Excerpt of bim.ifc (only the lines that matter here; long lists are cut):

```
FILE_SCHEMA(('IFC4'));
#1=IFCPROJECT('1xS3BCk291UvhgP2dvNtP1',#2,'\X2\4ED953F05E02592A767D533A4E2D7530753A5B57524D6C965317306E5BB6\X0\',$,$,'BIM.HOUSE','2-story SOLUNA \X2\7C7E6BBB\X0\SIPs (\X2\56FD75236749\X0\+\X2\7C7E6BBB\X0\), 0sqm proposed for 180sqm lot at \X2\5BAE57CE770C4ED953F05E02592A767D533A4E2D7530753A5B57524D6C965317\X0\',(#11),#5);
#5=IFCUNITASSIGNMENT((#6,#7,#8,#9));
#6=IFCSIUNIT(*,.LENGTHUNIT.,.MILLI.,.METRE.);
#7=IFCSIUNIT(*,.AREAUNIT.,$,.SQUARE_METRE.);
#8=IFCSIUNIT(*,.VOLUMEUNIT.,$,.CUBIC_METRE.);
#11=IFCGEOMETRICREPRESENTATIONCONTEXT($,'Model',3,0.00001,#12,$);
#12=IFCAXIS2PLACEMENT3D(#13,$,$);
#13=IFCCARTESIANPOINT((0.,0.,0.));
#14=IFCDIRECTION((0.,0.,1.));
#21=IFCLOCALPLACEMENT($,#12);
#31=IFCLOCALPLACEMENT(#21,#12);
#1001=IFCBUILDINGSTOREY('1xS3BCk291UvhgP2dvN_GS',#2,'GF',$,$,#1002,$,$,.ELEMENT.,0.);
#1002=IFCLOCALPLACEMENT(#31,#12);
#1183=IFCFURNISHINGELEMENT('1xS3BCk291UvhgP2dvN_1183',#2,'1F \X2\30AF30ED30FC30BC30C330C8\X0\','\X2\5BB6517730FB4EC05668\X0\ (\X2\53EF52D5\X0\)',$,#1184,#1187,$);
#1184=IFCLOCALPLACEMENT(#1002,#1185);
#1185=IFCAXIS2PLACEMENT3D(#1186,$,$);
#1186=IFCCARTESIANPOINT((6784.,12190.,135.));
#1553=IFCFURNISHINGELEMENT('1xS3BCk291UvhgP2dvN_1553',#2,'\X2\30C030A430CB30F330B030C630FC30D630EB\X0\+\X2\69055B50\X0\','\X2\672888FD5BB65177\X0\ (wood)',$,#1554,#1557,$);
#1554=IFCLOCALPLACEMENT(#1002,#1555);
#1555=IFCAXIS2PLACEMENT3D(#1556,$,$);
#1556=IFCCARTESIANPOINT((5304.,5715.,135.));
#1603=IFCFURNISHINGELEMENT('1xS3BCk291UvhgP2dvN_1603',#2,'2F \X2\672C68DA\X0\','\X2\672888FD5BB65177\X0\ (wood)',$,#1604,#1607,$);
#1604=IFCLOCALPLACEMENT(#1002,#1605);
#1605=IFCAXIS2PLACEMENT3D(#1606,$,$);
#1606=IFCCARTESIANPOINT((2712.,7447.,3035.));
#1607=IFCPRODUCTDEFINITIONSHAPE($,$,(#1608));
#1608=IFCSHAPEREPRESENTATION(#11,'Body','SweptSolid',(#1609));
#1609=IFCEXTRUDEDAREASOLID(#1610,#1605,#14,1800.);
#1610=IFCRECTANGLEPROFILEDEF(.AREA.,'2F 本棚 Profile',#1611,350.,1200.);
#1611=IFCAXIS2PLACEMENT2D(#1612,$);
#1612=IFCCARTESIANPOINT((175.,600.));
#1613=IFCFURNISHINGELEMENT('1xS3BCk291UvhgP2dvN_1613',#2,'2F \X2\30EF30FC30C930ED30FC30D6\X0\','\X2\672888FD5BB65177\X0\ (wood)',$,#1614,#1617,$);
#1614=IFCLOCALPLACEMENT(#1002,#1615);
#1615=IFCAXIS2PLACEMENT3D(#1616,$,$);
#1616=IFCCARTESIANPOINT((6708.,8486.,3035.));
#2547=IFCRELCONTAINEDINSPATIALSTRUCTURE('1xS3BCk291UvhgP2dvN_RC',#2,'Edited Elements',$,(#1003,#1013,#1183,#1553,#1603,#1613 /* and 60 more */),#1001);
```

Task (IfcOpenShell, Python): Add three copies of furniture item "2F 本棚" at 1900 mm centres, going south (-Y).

```python
import numpy as np
import ifcopenshell
import ifcopenshell.api.geometry
import ifcopenshell.api.root
import ifcopenshell.util.element
import ifcopenshell.util.placement
import ifcopenshell.util.unit

model = ifcopenshell.open("bim.ifc")
unit_scale = ifcopenshell.util.unit.calculate_unit_scale(model)


def reuse_history(source, copy):
    """copy_class also copies each property set's owner history, people and application; keep the originals."""
    for rel in copy.IsDefinedBy:
        if rel.is_a("IfcRelDefinesByProperties") and (history := rel.RelatingPropertyDefinition.OwnerHistory):
            rel.RelatingPropertyDefinition.OwnerHistory = source.OwnerHistory
            ifcopenshell.util.element.remove_deep2(model, history)


source = model.by_id(1603)
base = ifcopenshell.util.placement.get_local_placement(source.ObjectPlacement)
step = np.array([0.0, -1.0, 0.0]) * 1.9 / unit_scale

for i in range(1, 4):
    copy = ifcopenshell.api.root.copy_class(model, product=source)
    copy.Representation = ifcopenshell.util.element.copy_deep(
        model, source.Representation, exclude=["IfcGeometricRepresentationContext", "IfcRepresentationMap"]
    )
    reuse_history(source, copy)
    matrix = base.copy()
    matrix[:3, 3] += i * step
    print("added at", matrix[:3, 3].round(3) + 0.0)
    ifcopenshell.api.geometry.edit_object_placement(model, product=copy, matrix=matrix, is_si=False)

model.write("bim-out.ifc")
```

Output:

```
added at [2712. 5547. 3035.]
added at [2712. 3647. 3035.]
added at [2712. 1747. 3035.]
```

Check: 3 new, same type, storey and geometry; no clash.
